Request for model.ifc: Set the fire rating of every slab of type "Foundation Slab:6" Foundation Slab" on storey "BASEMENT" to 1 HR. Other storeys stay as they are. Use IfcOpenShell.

First a look at what the model holds.

```python
import ifcopenshell
import ifcopenshell.util.element

model = ifcopenshell.open("model.ifc")
print(model.schema)
storey = next(s for s in model.by_type("IfcBuildingStorey") if s.Name == "BASEMENT")
slabs = [e for e in ifcopenshell.util.element.get_decomposition(storey) if e.is_a("IfcSlab")]
seen = {}
for e in slabs:
    element_type = ifcopenshell.util.element.get_type(e)
    key = (element_type.Name if element_type != e and element_type else None, ifcopenshell.util.element.get_pset(e, "Pset_SlabCommon", "FireRating"))
    seen[key] = seen.get(key, 0) + 1
for (name, value), count in sorted(seen.items(), key=str):
    print(count, "x", name, "|", value)
```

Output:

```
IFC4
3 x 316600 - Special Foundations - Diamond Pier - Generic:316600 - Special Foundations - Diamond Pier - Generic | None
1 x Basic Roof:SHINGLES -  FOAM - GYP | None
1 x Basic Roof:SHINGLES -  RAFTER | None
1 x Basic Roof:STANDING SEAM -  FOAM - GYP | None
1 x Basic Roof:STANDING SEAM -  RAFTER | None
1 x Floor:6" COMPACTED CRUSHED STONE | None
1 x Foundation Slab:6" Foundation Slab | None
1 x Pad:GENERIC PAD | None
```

```python
import ifcopenshell
import ifcopenshell.api.pset
import ifcopenshell.util.element

model = ifcopenshell.open("model.ifc")

storey = next(s for s in model.by_type("IfcBuildingStorey") if s.Name == "BASEMENT")
slabs = [e for e in ifcopenshell.util.element.get_decomposition(storey) if e.is_a("IfcSlab")]

count = 0
for e in slabs:
    element_type = ifcopenshell.util.element.get_type(e)
    if element_type in (None, e) or element_type.Name != 'Foundation Slab:6" Foundation Slab':
        continue
    # add_pset returns the element's existing set when there is one.
    pset = ifcopenshell.api.pset.add_pset(model, product=e, name="Pset_SlabCommon")
    ifcopenshell.api.pset.edit_pset(model, pset=pset, properties={"FireRating": "1 HR"})
    count += 1

print(count, "slabs updated")

model.write("model-out.ifc")
```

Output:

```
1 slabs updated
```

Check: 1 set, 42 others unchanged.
